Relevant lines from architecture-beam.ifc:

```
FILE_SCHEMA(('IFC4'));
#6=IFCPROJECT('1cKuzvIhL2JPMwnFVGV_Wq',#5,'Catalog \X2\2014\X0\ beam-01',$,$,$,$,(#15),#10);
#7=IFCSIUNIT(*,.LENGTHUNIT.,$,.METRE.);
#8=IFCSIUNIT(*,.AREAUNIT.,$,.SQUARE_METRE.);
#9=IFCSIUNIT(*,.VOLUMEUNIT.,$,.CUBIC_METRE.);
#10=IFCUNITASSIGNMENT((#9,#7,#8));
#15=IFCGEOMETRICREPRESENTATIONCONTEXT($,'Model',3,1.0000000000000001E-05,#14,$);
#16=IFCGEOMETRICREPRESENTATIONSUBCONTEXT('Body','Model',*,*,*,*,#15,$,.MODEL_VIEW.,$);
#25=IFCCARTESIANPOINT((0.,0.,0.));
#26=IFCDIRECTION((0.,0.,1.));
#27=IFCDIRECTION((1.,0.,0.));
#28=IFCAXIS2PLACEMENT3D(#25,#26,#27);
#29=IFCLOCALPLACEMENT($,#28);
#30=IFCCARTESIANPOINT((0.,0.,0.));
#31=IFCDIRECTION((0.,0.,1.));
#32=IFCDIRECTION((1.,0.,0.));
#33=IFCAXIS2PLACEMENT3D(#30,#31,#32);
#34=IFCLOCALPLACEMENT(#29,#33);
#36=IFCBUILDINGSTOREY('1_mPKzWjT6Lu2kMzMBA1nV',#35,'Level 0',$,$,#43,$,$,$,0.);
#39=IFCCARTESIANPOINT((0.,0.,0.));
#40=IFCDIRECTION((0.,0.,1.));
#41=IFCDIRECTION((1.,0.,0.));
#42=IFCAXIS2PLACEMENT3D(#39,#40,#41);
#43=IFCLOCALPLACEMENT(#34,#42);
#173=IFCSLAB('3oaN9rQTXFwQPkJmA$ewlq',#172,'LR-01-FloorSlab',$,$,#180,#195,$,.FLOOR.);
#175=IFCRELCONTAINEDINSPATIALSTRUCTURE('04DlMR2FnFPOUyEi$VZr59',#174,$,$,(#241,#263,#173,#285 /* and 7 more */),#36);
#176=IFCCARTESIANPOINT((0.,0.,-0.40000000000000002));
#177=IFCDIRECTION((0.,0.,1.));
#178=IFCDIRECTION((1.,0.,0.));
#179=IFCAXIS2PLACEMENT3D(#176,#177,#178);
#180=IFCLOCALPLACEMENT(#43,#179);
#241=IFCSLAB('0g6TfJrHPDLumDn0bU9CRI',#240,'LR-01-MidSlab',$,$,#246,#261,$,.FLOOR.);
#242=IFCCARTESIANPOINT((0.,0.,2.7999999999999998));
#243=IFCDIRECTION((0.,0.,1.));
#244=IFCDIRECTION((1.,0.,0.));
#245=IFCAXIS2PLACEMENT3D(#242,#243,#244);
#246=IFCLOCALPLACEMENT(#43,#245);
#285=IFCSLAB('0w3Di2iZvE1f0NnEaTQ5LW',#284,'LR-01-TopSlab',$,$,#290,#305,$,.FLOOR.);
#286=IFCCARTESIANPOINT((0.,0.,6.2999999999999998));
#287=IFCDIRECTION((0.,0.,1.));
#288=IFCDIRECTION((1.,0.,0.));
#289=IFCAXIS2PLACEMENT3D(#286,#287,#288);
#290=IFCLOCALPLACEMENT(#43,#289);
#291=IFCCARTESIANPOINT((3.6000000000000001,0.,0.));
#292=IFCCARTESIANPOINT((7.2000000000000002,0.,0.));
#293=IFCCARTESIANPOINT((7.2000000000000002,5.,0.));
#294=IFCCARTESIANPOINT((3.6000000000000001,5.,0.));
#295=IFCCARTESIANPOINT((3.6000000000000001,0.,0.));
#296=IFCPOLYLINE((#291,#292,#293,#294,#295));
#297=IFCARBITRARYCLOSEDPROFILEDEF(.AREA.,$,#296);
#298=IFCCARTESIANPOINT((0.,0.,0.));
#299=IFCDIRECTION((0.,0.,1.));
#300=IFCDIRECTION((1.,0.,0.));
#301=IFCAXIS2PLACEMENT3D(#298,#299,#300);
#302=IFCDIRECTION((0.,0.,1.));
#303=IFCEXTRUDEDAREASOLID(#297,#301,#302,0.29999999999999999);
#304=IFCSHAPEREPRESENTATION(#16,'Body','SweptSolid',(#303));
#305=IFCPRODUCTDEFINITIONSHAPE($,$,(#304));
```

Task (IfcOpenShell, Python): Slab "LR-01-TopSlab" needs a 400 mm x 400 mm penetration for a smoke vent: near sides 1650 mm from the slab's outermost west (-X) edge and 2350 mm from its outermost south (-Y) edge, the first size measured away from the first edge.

```python
import numpy as np
import ifcopenshell
import ifcopenshell.api.feature
import ifcopenshell.api.geometry
import ifcopenshell.api.root
import ifcopenshell.geom
import ifcopenshell.util.placement
import ifcopenshell.util.representation
import ifcopenshell.util.shape
import ifcopenshell.util.unit

model = ifcopenshell.open("architecture-beam.ifc")
unit_scale = ifcopenshell.util.unit.calculate_unit_scale(model)
settings = ifcopenshell.geom.settings()


def volume(element):
    """Net volume in cubic metres, openings subtracted."""
    shape = ifcopenshell.geom.create_shape(settings, element)
    return ifcopenshell.util.shape.get_volume(shape.geometry)


slab = model.by_guid("0w3Di2iZvE1f0NnEaTQ5LW")
before = volume(slab)

# Extent in the slab's own axes, in metres. The edges named are its -X and -Y sides.
slab_shape = ifcopenshell.geom.create_shape(settings, slab)
vertices = ifcopenshell.util.shape.get_vertices(slab_shape.geometry)
x_min, y_min, bottom = vertices.min(axis=0)
top = vertices[:, 2].max()

opening = ifcopenshell.api.root.create_entity(model, ifc_class="IfcOpeningElement", name="Smoke vent opening", predefined_type="OPENING")
context = ifcopenshell.util.representation.get_context(model, "Model", "Body", "MODEL_VIEW")
width, depth = 0.4, 0.4
outline = [(0.0, 0.0), (width, 0.0), (width, depth), (0.0, depth), (0.0, 0.0)]
# Overshoot both faces by 50 mm so the cut is clean.
shape = ifcopenshell.api.geometry.add_slab_representation(
    model, context=context, depth=top - bottom + 0.1, polyline=outline
)
ifcopenshell.api.geometry.assign_representation(model, product=opening, representation=shape)

matrix = ifcopenshell.util.placement.get_local_placement(slab.ObjectPlacement)
matrix[:, 3] = matrix @ np.append(np.array([x_min + 1.65, y_min + 2.35, bottom - 0.05]) / unit_scale, 1.0)
ifcopenshell.api.geometry.edit_object_placement(model, product=opening, matrix=matrix, is_si=False)
ifcopenshell.api.feature.add_feature(model, feature=opening, element=slab)

after = volume(slab)

print(f"slab volume {before:.3f} -> {after:.3f} m3")

model.write("architecture-beam_updated.ifc")
```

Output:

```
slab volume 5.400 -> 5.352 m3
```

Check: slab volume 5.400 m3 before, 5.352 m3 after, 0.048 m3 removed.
